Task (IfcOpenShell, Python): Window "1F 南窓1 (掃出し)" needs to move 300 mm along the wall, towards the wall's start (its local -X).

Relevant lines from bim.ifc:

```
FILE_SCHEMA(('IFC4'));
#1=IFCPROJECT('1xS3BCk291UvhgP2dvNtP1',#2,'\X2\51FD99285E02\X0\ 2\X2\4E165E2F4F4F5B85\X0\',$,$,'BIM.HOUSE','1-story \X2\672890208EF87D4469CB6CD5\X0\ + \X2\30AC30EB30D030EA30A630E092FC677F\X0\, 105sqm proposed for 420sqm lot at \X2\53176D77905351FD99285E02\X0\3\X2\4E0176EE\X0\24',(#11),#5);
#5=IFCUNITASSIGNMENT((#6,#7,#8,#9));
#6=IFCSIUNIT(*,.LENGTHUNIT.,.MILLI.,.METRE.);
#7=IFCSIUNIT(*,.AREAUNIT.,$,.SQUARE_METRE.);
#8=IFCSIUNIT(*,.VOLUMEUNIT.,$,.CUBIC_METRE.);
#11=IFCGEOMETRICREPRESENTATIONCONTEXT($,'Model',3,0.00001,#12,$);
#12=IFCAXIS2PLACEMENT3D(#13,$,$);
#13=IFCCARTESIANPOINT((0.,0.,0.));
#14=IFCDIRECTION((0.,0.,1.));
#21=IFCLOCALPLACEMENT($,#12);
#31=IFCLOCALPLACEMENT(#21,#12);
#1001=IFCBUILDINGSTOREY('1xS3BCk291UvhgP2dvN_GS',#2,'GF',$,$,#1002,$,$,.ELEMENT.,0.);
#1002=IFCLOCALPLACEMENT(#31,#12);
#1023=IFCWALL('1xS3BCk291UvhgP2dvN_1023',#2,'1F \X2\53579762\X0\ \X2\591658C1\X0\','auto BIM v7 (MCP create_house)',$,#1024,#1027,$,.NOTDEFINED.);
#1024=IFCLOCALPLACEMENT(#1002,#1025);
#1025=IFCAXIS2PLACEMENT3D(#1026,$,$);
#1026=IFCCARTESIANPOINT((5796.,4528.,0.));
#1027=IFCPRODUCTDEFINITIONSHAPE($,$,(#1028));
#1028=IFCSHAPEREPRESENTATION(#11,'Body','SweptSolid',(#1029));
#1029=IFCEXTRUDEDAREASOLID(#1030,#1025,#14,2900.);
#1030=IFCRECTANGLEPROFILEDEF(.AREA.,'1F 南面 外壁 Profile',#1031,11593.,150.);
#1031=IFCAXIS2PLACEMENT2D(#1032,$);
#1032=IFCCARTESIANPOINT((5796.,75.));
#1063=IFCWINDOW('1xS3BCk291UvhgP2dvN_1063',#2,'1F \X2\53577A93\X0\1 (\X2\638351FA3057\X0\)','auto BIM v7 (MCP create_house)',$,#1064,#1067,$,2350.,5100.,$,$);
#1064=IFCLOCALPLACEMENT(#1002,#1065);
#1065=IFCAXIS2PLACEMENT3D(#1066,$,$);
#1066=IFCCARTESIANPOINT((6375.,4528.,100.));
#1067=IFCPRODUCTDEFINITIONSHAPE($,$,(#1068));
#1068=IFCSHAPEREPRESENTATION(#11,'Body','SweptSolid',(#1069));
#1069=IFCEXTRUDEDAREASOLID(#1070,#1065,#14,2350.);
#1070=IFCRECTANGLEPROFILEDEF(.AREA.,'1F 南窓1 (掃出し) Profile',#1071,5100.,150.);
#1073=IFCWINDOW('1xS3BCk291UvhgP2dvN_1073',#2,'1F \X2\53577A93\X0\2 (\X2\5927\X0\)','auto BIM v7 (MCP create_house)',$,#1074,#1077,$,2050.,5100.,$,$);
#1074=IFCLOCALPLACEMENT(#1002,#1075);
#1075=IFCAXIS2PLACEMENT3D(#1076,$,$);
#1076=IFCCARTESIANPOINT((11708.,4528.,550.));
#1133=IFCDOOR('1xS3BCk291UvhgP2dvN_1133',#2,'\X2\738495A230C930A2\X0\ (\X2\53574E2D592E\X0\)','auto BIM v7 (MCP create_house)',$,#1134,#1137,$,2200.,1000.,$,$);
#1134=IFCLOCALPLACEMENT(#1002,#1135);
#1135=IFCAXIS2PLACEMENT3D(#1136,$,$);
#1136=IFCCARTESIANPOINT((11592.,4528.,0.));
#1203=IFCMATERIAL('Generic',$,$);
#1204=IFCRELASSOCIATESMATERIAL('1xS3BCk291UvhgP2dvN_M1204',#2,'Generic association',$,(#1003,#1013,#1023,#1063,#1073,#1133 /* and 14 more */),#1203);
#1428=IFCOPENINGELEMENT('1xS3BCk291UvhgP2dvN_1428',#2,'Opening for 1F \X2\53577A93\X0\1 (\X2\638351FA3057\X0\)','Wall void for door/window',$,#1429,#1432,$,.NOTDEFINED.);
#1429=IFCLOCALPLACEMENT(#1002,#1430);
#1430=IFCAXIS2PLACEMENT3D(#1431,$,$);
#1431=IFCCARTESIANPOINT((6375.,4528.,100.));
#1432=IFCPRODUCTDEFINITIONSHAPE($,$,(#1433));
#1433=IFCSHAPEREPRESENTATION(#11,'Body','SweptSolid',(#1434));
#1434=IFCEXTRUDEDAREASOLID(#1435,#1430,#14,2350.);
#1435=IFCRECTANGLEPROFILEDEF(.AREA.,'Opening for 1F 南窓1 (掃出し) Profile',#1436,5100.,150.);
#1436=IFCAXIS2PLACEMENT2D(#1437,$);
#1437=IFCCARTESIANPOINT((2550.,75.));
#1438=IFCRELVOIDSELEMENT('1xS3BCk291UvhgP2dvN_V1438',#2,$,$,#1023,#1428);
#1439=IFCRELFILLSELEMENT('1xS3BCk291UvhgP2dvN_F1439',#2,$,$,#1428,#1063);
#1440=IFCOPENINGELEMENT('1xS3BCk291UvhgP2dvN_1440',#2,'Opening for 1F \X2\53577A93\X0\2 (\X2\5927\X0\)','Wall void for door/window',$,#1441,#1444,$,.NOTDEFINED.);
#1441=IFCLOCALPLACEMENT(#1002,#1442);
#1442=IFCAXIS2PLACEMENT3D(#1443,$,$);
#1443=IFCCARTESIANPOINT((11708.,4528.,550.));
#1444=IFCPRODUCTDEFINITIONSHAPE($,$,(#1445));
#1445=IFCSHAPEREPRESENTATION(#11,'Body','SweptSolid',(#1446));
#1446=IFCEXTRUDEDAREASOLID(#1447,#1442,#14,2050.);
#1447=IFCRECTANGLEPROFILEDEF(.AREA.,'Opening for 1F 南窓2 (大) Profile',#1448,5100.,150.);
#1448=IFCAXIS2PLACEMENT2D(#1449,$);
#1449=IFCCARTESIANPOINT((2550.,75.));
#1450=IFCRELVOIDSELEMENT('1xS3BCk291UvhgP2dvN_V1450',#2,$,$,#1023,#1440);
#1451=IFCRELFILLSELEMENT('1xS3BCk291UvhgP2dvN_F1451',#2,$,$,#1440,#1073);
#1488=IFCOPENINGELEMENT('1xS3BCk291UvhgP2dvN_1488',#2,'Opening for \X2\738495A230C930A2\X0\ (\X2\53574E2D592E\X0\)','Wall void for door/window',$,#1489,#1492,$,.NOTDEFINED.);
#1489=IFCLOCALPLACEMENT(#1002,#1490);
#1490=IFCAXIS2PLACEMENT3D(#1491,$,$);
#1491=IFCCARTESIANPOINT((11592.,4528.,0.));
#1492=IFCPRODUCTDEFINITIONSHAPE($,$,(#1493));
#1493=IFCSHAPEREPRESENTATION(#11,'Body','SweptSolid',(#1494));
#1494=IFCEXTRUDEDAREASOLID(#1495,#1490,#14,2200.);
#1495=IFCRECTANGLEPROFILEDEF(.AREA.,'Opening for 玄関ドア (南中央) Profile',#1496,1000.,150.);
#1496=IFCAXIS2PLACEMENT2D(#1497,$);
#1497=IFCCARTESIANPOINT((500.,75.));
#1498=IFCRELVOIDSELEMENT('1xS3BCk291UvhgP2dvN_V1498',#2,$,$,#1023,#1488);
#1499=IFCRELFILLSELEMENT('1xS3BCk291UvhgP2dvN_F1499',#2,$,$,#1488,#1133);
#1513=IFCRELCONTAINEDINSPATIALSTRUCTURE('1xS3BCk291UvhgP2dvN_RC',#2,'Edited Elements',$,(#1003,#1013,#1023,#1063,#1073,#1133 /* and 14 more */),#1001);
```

```python
import ifcopenshell
import ifcopenshell.api.geometry
import ifcopenshell.util.placement

model = ifcopenshell.open("bim.ifc")

window = model.by_guid("1xS3BCk291UvhgP2dvN_1063")
opening = window.FillsVoids[0].RelatingOpeningElement
wall = opening.VoidsElements[0].RelatingBuildingElement

wall_matrix = ifcopenshell.util.placement.get_local_placement(wall.ObjectPlacement)
shift = wall_matrix[:3, 0] * -300.0
before = ifcopenshell.util.placement.get_local_placement(window.ObjectPlacement)[:3, 3].copy()

# The window is not placed relative to its opening, so move both.
for product in (opening, window):
    matrix = ifcopenshell.util.placement.get_local_placement(product.ObjectPlacement)
    matrix[:3, 3] += shift
    ifcopenshell.api.geometry.edit_object_placement(model, product=product, matrix=matrix, is_si=False)

after = ifcopenshell.util.placement.get_local_placement(window.ObjectPlacement)[:3, 3]
print("window moved by", (after - before).round(3) + 0.0)

model.write("bim_rev.ifc")
```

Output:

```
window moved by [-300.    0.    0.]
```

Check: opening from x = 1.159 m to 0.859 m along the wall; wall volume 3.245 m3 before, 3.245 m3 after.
